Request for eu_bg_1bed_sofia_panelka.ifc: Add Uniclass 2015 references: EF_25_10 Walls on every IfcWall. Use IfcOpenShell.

First a look at what the model holds.

```python
import ifcopenshell

model = ifcopenshell.open("eu_bg_1bed_sofia_panelka.ifc")
print(model.schema)
print("classifications:", [c.Name for c in model.by_type("IfcClassification")])
for ifc_class in ("IfcDoor", "IfcRoof", "IfcStair", "IfcWall", "IfcWindow"):
    print(ifc_class, len(model.by_type(ifc_class)))
```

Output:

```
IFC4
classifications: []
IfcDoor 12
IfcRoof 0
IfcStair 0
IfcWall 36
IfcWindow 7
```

```python
import ifcopenshell
import ifcopenshell.api.classification

model = ifcopenshell.open("eu_bg_1bed_sofia_panelka.ifc")

system = ifcopenshell.api.classification.add_classification(model, classification="Uniclass 2015")

codes = {
    "IfcWall": ("EF_25_10", "Walls"),
}
for ifc_class, (code, name) in codes.items():
    products = model.by_type(ifc_class)
    ifcopenshell.api.classification.add_reference(
        model, products=products, classification=system, identification=code, name=name
    )
    print(code, len(products))

model.write("eu_bg_1bed_sofia_panelka_v2.ifc")
```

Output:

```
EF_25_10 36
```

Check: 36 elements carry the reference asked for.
